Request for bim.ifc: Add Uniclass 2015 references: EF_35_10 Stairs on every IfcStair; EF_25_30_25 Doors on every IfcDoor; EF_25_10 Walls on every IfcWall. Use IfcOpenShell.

First a look at what the model holds.

```python
import ifcopenshell

model = ifcopenshell.open("bim.ifc")
print(model.schema)
print("classifications:", [c.Name for c in model.by_type("IfcClassification")])
for ifc_class in ("IfcDoor", "IfcRoof", "IfcStair", "IfcWall", "IfcWindow"):
    print(ifc_class, len(model.by_type(ifc_class)))
```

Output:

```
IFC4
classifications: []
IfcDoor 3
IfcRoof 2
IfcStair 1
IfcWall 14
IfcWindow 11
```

```python
import ifcopenshell
import ifcopenshell.api.classification

model = ifcopenshell.open("bim.ifc")

system = ifcopenshell.api.classification.add_classification(model, classification="Uniclass 2015")

codes = {
    "IfcStair": ("EF_35_10", "Stairs"),
    "IfcDoor": ("EF_25_30_25", "Doors"),
    "IfcWall": ("EF_25_10", "Walls"),
}
for ifc_class, (code, name) in codes.items():
    products = model.by_type(ifc_class)
    ifcopenshell.api.classification.add_reference(
        model, products=products, classification=system, identification=code, name=name
    )
    print(code, len(products))

model.write("bim_v2.ifc")
```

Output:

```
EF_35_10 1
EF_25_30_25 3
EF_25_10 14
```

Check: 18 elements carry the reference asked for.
